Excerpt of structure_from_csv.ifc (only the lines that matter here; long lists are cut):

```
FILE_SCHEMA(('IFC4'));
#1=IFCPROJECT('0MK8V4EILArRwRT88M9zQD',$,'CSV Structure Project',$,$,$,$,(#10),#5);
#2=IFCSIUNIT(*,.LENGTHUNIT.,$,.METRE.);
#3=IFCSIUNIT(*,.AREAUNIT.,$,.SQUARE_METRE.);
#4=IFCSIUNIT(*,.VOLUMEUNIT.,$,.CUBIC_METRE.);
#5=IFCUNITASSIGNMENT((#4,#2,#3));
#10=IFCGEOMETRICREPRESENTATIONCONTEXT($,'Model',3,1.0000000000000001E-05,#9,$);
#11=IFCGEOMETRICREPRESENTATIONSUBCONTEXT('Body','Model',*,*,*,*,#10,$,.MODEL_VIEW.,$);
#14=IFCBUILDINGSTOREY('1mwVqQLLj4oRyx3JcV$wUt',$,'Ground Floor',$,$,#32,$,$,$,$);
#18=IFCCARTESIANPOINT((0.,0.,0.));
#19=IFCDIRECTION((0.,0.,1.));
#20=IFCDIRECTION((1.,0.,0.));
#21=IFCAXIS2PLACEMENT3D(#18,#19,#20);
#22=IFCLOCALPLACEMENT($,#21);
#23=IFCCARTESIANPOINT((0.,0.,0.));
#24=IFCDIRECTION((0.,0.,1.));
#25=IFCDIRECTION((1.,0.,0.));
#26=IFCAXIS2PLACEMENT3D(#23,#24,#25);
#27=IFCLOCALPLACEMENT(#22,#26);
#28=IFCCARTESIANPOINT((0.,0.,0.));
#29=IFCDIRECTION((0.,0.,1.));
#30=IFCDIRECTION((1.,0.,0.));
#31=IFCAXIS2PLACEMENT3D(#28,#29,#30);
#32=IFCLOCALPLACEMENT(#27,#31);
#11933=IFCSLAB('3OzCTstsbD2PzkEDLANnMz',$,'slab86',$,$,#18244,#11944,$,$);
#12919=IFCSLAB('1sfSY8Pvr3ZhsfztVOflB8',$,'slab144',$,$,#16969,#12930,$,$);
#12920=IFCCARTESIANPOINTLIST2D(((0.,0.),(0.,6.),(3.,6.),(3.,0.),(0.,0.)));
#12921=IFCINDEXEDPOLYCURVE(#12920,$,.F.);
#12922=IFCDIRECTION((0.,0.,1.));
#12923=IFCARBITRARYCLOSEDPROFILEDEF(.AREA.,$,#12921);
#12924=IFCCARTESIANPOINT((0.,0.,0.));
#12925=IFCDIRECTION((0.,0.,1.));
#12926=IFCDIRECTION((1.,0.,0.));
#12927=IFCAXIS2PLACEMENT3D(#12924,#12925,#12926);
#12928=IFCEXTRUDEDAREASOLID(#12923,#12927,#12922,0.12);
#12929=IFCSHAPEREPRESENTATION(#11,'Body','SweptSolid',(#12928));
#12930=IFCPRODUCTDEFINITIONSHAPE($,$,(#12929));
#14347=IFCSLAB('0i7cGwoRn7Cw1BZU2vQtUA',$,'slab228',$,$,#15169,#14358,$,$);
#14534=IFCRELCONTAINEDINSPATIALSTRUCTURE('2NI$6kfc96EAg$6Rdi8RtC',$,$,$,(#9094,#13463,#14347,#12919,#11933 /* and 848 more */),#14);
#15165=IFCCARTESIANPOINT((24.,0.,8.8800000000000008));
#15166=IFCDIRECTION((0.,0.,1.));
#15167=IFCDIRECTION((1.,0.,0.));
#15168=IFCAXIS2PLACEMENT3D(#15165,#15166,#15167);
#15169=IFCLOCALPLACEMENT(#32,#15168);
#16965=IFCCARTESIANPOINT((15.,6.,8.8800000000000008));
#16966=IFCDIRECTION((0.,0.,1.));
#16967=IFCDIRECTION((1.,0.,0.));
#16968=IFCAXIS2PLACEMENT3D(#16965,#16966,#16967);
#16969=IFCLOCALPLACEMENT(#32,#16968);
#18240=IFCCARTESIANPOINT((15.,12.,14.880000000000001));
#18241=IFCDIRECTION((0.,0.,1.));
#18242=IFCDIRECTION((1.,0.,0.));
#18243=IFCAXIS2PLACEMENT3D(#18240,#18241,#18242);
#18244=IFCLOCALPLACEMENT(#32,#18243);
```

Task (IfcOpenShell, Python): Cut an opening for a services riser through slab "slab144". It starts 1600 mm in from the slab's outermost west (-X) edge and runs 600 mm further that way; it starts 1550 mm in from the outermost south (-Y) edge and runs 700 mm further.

```python
import numpy as np
import ifcopenshell
import ifcopenshell.api.feature
import ifcopenshell.api.geometry
import ifcopenshell.api.root
import ifcopenshell.geom
import ifcopenshell.util.placement
import ifcopenshell.util.representation
import ifcopenshell.util.shape
import ifcopenshell.util.unit

model = ifcopenshell.open("structure_from_csv.ifc")
unit_scale = ifcopenshell.util.unit.calculate_unit_scale(model)
settings = ifcopenshell.geom.settings()


def volume(element):
    """Net volume in cubic metres, openings subtracted."""
    shape = ifcopenshell.geom.create_shape(settings, element)
    return ifcopenshell.util.shape.get_volume(shape.geometry)


slab = model.by_id(12919)
before = volume(slab)

# Extent in the slab's own axes, in metres. The edges named are its -X and -Y sides.
slab_shape = ifcopenshell.geom.create_shape(settings, slab)
vertices = ifcopenshell.util.shape.get_vertices(slab_shape.geometry)
x_min, y_min, bottom = vertices.min(axis=0)
top = vertices[:, 2].max()

opening = ifcopenshell.api.root.create_entity(model, ifc_class="IfcOpeningElement", name="Services riser opening", predefined_type="OPENING")
context = ifcopenshell.util.representation.get_context(model, "Model", "Body", "MODEL_VIEW")
width, depth = 0.6, 0.7
outline = [(0.0, 0.0), (width, 0.0), (width, depth), (0.0, depth), (0.0, 0.0)]
# Overshoot both faces by 50 mm so the cut is clean.
shape = ifcopenshell.api.geometry.add_slab_representation(
    model, context=context, depth=top - bottom + 0.1, polyline=outline
)
ifcopenshell.api.geometry.assign_representation(model, product=opening, representation=shape)

matrix = ifcopenshell.util.placement.get_local_placement(slab.ObjectPlacement)
matrix[:, 3] = matrix @ np.append(np.array([x_min + 1.6, y_min + 1.55, bottom - 0.05]) / unit_scale, 1.0)
ifcopenshell.api.geometry.edit_object_placement(model, product=opening, matrix=matrix, is_si=False)
ifcopenshell.api.feature.add_feature(model, feature=opening, element=slab)

after = volume(slab)

print(f"slab volume {before:.3f} -> {after:.3f} m3")

model.write("structure_from_csv_edited.ifc")
```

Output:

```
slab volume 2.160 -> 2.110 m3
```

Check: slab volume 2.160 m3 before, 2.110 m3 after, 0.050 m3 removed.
